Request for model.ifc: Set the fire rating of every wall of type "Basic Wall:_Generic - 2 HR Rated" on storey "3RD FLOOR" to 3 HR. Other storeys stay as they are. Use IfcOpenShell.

First a look at what the model holds.

```python
import ifcopenshell
import ifcopenshell.util.element

model = ifcopenshell.open("model.ifc")
print(model.schema)
storey = next(s for s in model.by_type("IfcBuildingStorey") if s.Name == "3RD FLOOR")
walls = [e for e in ifcopenshell.util.element.get_decomposition(storey) if e.is_a("IfcWall")]
seen = {}
for e in walls:
    element_type = ifcopenshell.util.element.get_type(e)
    key = (element_type.Name if element_type != e and element_type else None, ifcopenshell.util.element.get_pset(e, "Pset_WallCommon", "FireRating"))
    seen[key] = seen.get(key, 0) + 1
for (name, value), count in sorted(seen.items(), key=str):
    print(count, "x", name, "|", value)
```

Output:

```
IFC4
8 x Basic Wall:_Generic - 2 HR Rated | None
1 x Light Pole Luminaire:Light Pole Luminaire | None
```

```python
import ifcopenshell
import ifcopenshell.api.pset
import ifcopenshell.util.element

model = ifcopenshell.open("model.ifc")

storey = next(s for s in model.by_type("IfcBuildingStorey") if s.Name == "3RD FLOOR")
walls = [e for e in ifcopenshell.util.element.get_decomposition(storey) if e.is_a("IfcWall")]

count = 0
for e in walls:
    element_type = ifcopenshell.util.element.get_type(e)
    if element_type in (None, e) or element_type.Name != "Basic Wall:_Generic - 2 HR Rated":
        continue
    # add_pset returns the element's existing set when there is one.
    pset = ifcopenshell.api.pset.add_pset(model, product=e, name="Pset_WallCommon")
    ifcopenshell.api.pset.edit_pset(model, pset=pset, properties={"FireRating": "3 HR"})
    count += 1

print(count, "walls updated")

model.write("model_updated.ifc")
```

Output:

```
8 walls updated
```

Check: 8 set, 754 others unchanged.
